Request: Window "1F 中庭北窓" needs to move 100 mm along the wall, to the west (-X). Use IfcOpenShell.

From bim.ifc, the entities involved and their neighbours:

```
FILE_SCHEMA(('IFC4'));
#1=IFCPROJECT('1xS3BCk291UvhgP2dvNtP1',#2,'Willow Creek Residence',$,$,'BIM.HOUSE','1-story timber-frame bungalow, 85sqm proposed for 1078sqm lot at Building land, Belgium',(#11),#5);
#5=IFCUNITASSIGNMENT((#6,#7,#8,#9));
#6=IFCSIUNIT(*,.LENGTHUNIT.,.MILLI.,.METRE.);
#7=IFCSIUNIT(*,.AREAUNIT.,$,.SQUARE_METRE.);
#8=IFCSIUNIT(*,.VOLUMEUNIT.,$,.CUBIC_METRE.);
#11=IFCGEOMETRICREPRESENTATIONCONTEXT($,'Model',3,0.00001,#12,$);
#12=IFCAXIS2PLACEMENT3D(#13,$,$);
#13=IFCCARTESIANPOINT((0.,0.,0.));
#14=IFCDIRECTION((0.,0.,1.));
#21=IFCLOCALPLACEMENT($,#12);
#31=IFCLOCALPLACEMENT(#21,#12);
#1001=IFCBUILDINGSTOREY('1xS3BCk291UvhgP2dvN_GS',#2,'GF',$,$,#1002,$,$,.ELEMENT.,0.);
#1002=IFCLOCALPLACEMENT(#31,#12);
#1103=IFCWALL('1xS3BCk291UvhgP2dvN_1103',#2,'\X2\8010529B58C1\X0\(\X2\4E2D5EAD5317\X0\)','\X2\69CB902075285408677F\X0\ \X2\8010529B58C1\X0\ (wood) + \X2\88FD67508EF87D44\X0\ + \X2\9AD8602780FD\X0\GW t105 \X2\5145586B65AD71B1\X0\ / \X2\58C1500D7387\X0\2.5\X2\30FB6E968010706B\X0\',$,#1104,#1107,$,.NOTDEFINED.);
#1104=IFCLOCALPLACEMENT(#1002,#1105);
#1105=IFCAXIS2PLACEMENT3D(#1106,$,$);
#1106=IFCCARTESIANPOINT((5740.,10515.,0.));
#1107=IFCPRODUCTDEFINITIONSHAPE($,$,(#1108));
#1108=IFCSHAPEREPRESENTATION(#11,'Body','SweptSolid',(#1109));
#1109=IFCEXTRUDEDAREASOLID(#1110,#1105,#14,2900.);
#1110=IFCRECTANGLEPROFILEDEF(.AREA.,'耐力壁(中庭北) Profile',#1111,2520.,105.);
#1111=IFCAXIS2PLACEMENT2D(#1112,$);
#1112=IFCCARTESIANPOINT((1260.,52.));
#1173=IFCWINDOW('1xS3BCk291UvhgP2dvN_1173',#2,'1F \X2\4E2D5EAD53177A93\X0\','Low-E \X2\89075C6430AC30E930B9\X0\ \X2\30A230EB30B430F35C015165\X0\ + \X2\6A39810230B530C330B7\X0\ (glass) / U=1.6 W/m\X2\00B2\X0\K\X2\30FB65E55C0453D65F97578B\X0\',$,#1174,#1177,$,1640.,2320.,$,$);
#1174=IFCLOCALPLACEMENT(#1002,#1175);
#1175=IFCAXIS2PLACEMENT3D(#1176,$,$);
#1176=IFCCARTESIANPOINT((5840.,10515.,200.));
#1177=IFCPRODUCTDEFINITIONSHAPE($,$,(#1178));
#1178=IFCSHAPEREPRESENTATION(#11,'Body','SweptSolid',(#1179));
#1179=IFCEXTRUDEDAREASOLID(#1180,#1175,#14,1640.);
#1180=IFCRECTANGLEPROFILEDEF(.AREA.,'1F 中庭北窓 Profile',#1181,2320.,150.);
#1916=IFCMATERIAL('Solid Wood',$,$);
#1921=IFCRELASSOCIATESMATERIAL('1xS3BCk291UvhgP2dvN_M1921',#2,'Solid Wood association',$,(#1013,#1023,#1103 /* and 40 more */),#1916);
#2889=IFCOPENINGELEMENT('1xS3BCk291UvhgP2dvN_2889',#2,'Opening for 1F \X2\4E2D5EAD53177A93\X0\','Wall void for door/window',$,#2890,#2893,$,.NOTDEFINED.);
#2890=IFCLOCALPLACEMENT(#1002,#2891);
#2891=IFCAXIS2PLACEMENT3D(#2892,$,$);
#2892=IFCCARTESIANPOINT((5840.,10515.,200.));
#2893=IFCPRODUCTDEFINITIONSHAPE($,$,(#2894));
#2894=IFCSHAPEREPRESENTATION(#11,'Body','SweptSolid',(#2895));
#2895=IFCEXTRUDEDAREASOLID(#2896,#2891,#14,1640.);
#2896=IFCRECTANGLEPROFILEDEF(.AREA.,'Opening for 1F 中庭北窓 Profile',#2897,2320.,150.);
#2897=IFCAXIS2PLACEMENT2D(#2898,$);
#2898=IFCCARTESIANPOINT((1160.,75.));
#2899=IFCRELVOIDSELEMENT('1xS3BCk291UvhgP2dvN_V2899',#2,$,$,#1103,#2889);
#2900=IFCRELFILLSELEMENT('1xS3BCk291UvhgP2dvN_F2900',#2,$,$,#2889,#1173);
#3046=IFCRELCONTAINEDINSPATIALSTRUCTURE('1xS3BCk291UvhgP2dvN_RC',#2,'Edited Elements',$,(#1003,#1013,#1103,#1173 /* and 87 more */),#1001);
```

```python
import ifcopenshell
import ifcopenshell.api.geometry
import ifcopenshell.util.placement
import ifcopenshell.util.unit

model = ifcopenshell.open("bim.ifc")
unit_scale = ifcopenshell.util.unit.calculate_unit_scale(model)

window = model.by_id(1173)
opening = window.FillsVoids[0].RelatingOpeningElement
wall = opening.VoidsElements[0].RelatingBuildingElement

wall_matrix = ifcopenshell.util.placement.get_local_placement(wall.ObjectPlacement)
shift = wall_matrix[:3, 0] * -0.1 / unit_scale
before = ifcopenshell.util.placement.get_local_placement(window.ObjectPlacement)[:3, 3].copy()

# The window is not placed relative to its opening, so move both.
for product in (opening, window):
    matrix = ifcopenshell.util.placement.get_local_placement(product.ObjectPlacement)
    matrix[:3, 3] += shift
    ifcopenshell.api.geometry.edit_object_placement(model, product=product, matrix=matrix, is_si=False)

after = ifcopenshell.util.placement.get_local_placement(window.ObjectPlacement)[:3, 3]
print("window moved by", (after - before).round(3) + 0.0)

model.write("bim_edited.ifc")
```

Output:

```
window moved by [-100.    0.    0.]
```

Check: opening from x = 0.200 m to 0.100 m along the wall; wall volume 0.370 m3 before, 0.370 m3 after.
